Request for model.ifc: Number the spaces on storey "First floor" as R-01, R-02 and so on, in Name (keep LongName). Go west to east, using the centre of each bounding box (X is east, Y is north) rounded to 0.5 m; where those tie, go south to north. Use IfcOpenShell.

First a look at what the model holds.

```python
import ifcopenshell
import ifcopenshell.util.element
import ifcopenshell.util.placement

model = ifcopenshell.open("model.ifc")
print(model.schema)
storey = next(s for s in model.by_type("IfcBuildingStorey") if s.Name == "First floor")
spaces = [e for e in ifcopenshell.util.element.get_decomposition(storey) if e.is_a("IfcSpace")]
for e in sorted(spaces, key=lambda e: e.id()):
    origin = ifcopenshell.util.placement.get_local_placement(e.ObjectPlacement)[:3, 3]
    print(e.id(), e.Name, e.LongName, origin.round(2) + 0.0, sep=" | ")
```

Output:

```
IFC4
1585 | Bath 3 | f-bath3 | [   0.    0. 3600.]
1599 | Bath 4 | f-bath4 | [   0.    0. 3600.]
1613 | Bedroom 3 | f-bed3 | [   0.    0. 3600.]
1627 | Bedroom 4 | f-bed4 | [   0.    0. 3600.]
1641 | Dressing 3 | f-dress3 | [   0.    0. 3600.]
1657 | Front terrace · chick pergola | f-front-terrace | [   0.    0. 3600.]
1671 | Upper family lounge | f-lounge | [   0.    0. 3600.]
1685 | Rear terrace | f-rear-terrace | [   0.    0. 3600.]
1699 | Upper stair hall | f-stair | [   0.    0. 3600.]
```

```python
import ifcopenshell
import ifcopenshell.geom
import ifcopenshell.util.element
import ifcopenshell.util.shape

model = ifcopenshell.open("model.ifc")
settings = ifcopenshell.geom.settings()
settings.set("use-world-coords", True)


def centre(element):
    shape = ifcopenshell.geom.create_shape(settings, element)
    return ifcopenshell.util.shape.get_bbox_centroid(shape.geometry)


storey = next(s for s in model.by_type("IfcBuildingStorey") if s.Name == "First floor")
spaces = [e for e in ifcopenshell.util.element.get_decomposition(storey) if e.is_a("IfcSpace")]

# Insertion points can sit at a corner or the storey origin, so sort by the geometry (in metres).
centres = {e: centre(e) for e in spaces}
spaces.sort(key=lambda e: (round(centres[e][0] / 0.5), centres[e][1]))

for i, e in enumerate(spaces, start=1):
    number = f"R-{i:02d}"
    e.Name = number
    print(e.id(), number)

model.write("model_v2.ifc")
```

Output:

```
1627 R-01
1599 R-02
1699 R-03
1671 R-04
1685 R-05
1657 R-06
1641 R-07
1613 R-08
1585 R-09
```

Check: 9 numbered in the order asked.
